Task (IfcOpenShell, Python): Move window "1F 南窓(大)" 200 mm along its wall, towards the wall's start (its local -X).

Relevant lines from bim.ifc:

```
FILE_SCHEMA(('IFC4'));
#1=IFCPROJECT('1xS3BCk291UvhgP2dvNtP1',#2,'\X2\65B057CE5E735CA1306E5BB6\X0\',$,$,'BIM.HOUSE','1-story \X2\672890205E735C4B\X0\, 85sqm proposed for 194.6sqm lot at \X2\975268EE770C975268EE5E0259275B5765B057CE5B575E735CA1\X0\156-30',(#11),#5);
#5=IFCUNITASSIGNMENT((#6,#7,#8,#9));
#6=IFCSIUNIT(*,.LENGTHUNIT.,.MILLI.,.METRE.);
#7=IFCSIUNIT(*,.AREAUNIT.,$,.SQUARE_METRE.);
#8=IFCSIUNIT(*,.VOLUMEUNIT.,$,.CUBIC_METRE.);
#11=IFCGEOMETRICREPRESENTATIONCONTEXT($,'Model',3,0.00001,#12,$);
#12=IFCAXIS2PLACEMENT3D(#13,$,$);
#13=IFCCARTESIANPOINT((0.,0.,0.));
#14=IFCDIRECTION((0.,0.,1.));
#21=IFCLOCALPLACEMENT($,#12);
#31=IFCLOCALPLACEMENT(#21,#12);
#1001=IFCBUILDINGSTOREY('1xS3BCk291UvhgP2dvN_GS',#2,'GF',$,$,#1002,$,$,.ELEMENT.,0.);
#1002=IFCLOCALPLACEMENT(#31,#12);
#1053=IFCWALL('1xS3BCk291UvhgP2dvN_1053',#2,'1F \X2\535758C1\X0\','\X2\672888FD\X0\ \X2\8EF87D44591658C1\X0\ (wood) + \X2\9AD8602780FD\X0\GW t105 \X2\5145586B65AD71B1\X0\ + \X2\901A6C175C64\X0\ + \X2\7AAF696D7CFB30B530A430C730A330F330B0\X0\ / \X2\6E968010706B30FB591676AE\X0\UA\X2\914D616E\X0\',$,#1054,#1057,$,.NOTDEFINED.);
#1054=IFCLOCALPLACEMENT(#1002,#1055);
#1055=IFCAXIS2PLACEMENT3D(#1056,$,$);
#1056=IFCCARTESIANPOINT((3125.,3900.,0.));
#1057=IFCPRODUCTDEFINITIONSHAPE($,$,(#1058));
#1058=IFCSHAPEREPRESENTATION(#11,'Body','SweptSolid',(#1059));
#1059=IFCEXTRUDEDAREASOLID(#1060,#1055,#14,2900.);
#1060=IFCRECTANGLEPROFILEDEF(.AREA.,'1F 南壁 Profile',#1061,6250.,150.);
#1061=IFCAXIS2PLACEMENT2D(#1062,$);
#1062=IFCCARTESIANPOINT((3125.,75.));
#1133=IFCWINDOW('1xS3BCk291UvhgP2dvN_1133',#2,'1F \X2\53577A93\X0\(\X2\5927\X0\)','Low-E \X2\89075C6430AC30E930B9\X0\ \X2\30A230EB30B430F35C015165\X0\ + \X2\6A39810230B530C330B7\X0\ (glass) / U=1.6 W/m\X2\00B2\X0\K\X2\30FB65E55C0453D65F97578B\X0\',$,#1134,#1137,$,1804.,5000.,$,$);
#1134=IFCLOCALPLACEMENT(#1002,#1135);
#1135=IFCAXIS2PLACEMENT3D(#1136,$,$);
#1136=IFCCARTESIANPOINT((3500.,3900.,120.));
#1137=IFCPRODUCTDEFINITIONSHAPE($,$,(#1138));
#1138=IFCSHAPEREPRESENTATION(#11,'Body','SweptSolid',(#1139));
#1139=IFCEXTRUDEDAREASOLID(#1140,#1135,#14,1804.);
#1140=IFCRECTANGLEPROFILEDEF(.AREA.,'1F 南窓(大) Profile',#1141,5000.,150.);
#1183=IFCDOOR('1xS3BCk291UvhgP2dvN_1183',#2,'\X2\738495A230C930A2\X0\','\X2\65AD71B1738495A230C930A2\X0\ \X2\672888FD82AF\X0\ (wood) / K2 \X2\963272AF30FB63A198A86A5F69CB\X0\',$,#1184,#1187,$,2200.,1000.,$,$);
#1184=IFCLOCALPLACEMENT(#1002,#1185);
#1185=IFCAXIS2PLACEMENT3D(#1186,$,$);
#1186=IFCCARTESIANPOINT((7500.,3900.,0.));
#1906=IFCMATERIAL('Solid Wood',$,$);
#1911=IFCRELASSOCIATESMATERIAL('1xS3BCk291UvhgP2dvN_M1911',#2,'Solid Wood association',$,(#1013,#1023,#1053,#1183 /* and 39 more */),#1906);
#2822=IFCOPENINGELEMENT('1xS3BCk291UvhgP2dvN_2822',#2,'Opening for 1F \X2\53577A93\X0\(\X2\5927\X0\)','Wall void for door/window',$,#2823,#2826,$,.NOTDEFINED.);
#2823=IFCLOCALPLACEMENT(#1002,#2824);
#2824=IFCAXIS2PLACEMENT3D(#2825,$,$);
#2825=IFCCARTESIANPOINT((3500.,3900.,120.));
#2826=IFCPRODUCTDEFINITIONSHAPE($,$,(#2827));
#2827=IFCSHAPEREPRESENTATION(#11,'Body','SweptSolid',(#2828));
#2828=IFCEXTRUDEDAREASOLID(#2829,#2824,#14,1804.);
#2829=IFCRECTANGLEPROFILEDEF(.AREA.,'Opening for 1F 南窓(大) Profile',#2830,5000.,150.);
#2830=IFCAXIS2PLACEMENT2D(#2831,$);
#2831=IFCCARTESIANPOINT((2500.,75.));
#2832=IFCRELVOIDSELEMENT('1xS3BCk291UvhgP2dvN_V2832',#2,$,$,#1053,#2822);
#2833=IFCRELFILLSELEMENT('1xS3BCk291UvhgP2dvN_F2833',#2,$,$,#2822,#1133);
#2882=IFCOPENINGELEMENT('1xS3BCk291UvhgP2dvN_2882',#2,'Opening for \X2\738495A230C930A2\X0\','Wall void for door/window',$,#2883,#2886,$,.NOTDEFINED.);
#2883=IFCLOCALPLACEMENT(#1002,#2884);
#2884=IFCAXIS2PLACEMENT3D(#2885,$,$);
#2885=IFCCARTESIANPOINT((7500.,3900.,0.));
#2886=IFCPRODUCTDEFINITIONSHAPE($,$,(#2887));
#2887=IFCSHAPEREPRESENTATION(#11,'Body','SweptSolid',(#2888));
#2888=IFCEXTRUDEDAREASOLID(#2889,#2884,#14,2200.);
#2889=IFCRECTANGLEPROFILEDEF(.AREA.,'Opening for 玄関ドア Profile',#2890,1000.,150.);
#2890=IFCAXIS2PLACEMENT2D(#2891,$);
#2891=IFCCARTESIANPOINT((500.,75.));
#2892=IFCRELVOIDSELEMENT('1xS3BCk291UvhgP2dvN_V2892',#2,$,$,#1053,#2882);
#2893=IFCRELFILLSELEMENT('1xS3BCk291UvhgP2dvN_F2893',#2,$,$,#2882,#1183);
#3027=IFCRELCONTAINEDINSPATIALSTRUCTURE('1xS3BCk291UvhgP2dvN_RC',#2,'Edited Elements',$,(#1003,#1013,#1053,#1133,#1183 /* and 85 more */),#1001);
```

```python
import ifcopenshell
import ifcopenshell.api.geometry
import ifcopenshell.util.placement

model = ifcopenshell.open("bim.ifc")

window = model.by_guid("1xS3BCk291UvhgP2dvN_1133")
opening = window.FillsVoids[0].RelatingOpeningElement
wall = opening.VoidsElements[0].RelatingBuildingElement

wall_matrix = ifcopenshell.util.placement.get_local_placement(wall.ObjectPlacement)
shift = wall_matrix[:3, 0] * -200.0
before = ifcopenshell.util.placement.get_local_placement(window.ObjectPlacement)[:3, 3].copy()

# The window is not placed relative to its opening, so move both.
for product in (opening, window):
    matrix = ifcopenshell.util.placement.get_local_placement(product.ObjectPlacement)
    matrix[:3, 3] += shift
    ifcopenshell.api.geometry.edit_object_placement(model, product=product, matrix=matrix, is_si=False)

after = ifcopenshell.util.placement.get_local_placement(window.ObjectPlacement)[:3, 3]
print("window moved by", (after - before).round(3) + 0.0)

model.write("bim_rev.ifc")
```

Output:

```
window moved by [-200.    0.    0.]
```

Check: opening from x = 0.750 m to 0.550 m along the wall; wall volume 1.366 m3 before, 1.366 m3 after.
